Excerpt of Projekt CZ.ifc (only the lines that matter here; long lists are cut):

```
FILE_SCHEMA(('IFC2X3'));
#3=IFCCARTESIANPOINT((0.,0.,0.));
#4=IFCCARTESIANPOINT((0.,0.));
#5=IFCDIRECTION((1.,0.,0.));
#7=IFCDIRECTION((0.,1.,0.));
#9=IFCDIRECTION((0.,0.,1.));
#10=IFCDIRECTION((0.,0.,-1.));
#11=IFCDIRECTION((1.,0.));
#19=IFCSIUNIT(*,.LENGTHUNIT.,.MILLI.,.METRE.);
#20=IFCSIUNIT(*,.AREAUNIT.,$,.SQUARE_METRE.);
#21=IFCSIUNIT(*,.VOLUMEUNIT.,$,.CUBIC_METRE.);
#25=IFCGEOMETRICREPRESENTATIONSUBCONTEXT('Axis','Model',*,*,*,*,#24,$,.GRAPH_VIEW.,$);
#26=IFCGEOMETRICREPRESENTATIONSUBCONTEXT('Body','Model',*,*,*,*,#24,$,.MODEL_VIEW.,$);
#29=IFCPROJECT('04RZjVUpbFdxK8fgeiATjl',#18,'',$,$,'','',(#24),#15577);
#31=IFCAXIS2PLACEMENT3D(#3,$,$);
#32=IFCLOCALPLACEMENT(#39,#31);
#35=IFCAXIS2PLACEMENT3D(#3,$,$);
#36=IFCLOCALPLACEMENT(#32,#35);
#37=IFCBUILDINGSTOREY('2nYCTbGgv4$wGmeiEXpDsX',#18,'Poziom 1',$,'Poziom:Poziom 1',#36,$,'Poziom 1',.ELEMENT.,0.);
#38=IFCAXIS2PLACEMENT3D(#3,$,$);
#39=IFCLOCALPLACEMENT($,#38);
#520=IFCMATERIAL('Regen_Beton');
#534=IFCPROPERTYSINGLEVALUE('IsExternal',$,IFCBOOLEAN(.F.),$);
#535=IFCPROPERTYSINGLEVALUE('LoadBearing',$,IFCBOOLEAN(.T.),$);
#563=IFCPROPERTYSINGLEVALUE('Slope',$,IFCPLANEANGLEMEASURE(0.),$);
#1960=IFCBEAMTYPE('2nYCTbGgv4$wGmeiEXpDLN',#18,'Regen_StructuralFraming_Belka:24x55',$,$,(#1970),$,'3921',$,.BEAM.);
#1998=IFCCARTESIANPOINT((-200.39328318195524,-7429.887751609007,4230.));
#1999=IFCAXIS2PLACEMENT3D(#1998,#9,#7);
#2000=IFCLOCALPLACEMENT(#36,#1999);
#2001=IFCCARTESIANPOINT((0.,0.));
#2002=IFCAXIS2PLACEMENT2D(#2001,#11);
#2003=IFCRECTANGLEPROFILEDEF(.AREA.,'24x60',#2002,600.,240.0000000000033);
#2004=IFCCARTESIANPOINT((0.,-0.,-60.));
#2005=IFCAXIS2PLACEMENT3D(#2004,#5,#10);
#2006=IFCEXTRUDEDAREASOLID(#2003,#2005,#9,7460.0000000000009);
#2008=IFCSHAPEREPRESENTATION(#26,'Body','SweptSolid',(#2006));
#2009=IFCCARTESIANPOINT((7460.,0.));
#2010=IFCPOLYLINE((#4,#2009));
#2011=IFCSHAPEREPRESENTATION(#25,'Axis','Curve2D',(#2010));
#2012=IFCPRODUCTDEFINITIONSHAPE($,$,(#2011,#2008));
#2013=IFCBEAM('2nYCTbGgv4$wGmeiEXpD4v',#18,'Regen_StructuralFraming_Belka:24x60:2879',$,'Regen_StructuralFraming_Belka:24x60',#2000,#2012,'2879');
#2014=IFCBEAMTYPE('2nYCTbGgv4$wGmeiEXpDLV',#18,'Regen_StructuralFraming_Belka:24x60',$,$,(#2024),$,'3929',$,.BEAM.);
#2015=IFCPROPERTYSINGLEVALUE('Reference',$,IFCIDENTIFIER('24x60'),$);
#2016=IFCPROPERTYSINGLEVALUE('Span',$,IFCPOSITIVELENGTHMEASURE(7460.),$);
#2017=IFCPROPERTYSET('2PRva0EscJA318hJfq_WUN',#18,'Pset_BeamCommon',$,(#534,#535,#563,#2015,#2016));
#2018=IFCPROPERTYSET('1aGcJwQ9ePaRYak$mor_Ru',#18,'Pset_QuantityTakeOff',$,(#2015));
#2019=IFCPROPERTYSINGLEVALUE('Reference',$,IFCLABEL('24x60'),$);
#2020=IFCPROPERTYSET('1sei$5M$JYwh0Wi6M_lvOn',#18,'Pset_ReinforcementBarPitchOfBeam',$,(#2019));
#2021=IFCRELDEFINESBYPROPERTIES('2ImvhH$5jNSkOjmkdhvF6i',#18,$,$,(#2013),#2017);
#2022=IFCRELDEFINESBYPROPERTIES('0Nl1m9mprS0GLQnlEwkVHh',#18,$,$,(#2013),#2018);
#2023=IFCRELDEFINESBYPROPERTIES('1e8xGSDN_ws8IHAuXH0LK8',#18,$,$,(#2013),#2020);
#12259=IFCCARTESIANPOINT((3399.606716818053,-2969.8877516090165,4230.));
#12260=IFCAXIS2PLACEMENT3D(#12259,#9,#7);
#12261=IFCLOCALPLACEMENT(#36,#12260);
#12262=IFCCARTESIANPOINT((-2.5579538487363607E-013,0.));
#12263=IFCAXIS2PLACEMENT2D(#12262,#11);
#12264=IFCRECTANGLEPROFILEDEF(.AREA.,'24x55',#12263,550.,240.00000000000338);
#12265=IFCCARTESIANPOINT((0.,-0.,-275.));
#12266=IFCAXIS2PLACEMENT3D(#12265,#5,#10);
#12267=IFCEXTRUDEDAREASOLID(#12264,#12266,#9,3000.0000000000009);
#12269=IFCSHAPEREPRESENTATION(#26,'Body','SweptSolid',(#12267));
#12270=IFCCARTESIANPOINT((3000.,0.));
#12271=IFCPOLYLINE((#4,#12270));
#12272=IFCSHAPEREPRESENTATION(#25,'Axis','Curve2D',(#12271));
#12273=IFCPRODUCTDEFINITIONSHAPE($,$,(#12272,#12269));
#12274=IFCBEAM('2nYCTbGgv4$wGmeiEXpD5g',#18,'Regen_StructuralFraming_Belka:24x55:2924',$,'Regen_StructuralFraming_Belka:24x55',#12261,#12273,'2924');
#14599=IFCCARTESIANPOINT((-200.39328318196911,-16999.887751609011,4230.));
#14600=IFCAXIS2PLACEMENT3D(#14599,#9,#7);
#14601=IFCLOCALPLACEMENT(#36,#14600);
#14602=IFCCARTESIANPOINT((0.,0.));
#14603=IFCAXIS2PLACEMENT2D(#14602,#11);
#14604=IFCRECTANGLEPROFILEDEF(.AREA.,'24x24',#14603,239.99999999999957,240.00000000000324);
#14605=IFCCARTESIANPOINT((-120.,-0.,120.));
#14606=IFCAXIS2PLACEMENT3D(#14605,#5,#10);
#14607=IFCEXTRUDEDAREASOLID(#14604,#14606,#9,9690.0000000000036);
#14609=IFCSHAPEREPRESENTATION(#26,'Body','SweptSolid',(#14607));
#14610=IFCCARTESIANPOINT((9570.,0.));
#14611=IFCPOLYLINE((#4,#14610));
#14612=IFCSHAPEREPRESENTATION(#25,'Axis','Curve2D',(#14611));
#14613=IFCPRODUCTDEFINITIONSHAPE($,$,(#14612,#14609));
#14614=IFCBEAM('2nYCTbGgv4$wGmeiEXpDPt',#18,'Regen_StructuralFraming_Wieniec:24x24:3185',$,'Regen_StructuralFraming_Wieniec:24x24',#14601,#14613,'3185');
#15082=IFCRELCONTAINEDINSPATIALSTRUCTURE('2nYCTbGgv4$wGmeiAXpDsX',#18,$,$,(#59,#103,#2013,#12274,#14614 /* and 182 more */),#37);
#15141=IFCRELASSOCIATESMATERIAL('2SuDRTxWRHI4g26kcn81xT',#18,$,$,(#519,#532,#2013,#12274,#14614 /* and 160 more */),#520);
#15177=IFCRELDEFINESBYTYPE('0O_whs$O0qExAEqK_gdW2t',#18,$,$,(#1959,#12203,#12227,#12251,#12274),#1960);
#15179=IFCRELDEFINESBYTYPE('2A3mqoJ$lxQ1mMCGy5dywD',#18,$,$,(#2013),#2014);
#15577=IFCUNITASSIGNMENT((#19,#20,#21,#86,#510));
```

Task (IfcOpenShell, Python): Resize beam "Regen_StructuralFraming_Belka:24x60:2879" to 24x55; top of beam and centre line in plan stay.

```python
import ifcopenshell
import ifcopenshell.api.pset
import ifcopenshell.api.type
import ifcopenshell.util.element
import ifcopenshell.util.representation

model = ifcopenshell.open("Projekt CZ.ifc")

member = model.by_id(2013)
source = next(p for p in model.by_type("IfcRectangleProfileDef") if p.ProfileName == "24x55")

body = ifcopenshell.util.representation.get_representation(member, "Model", "Body")
solid = body.Items[0]
old_profile = solid.SweptArea

# Copy the section's sizes but keep this member's own profile position.
profile = ifcopenshell.util.element.copy(model, source)
# Profiles are centred, so shift by half the change in depth to hold the top.
shift = (old_profile.XDim - profile.XDim) / 2
x, y = old_profile.Position.Location.Coordinates
up = (-1.0, 0.0)  # upwards, in the solid's own plane
location = model.createIfcCartesianPoint((x + up[0] * shift, y + up[1] * shift))
profile.Position = model.createIfcAxis2Placement2D(location, old_profile.Position.RefDirection)
solid.SweptArea = profile
if not model.get_total_inverses(old_profile):
    ifcopenshell.util.element.remove_deep2(model, old_profile)

new_type = model.by_id(1960)
ifcopenshell.api.type.assign_type(
    model, related_objects=[member], relating_type=new_type, should_map_representations=False
)
member.Name = member.Name.replace("24x60", "24x55")
member.ObjectType = "Regen_StructuralFraming_Belka:24x55"
pset = model.by_id(ifcopenshell.util.element.get_pset(member, "Pset_BeamCommon", should_inherit=False)["id"])
ifcopenshell.api.pset.edit_pset(model, pset=pset, properties={"Reference": "24x55"})
pset = model.by_id(ifcopenshell.util.element.get_pset(member, "Pset_QuantityTakeOff", should_inherit=False)["id"])
ifcopenshell.api.pset.edit_pset(model, pset=pset, properties={"Reference": "24x55"})
pset = model.by_id(ifcopenshell.util.element.get_pset(member, "Pset_ReinforcementBarPitchOfBeam", should_inherit=False)["id"])
ifcopenshell.api.pset.edit_pset(model, pset=pset, properties={"Reference": "24x55"})

print(solid.SweptArea)

model.write("Projekt CZ_rev.ifc")
```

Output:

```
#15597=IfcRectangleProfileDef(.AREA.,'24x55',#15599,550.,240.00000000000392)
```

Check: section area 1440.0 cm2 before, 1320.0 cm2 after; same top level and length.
